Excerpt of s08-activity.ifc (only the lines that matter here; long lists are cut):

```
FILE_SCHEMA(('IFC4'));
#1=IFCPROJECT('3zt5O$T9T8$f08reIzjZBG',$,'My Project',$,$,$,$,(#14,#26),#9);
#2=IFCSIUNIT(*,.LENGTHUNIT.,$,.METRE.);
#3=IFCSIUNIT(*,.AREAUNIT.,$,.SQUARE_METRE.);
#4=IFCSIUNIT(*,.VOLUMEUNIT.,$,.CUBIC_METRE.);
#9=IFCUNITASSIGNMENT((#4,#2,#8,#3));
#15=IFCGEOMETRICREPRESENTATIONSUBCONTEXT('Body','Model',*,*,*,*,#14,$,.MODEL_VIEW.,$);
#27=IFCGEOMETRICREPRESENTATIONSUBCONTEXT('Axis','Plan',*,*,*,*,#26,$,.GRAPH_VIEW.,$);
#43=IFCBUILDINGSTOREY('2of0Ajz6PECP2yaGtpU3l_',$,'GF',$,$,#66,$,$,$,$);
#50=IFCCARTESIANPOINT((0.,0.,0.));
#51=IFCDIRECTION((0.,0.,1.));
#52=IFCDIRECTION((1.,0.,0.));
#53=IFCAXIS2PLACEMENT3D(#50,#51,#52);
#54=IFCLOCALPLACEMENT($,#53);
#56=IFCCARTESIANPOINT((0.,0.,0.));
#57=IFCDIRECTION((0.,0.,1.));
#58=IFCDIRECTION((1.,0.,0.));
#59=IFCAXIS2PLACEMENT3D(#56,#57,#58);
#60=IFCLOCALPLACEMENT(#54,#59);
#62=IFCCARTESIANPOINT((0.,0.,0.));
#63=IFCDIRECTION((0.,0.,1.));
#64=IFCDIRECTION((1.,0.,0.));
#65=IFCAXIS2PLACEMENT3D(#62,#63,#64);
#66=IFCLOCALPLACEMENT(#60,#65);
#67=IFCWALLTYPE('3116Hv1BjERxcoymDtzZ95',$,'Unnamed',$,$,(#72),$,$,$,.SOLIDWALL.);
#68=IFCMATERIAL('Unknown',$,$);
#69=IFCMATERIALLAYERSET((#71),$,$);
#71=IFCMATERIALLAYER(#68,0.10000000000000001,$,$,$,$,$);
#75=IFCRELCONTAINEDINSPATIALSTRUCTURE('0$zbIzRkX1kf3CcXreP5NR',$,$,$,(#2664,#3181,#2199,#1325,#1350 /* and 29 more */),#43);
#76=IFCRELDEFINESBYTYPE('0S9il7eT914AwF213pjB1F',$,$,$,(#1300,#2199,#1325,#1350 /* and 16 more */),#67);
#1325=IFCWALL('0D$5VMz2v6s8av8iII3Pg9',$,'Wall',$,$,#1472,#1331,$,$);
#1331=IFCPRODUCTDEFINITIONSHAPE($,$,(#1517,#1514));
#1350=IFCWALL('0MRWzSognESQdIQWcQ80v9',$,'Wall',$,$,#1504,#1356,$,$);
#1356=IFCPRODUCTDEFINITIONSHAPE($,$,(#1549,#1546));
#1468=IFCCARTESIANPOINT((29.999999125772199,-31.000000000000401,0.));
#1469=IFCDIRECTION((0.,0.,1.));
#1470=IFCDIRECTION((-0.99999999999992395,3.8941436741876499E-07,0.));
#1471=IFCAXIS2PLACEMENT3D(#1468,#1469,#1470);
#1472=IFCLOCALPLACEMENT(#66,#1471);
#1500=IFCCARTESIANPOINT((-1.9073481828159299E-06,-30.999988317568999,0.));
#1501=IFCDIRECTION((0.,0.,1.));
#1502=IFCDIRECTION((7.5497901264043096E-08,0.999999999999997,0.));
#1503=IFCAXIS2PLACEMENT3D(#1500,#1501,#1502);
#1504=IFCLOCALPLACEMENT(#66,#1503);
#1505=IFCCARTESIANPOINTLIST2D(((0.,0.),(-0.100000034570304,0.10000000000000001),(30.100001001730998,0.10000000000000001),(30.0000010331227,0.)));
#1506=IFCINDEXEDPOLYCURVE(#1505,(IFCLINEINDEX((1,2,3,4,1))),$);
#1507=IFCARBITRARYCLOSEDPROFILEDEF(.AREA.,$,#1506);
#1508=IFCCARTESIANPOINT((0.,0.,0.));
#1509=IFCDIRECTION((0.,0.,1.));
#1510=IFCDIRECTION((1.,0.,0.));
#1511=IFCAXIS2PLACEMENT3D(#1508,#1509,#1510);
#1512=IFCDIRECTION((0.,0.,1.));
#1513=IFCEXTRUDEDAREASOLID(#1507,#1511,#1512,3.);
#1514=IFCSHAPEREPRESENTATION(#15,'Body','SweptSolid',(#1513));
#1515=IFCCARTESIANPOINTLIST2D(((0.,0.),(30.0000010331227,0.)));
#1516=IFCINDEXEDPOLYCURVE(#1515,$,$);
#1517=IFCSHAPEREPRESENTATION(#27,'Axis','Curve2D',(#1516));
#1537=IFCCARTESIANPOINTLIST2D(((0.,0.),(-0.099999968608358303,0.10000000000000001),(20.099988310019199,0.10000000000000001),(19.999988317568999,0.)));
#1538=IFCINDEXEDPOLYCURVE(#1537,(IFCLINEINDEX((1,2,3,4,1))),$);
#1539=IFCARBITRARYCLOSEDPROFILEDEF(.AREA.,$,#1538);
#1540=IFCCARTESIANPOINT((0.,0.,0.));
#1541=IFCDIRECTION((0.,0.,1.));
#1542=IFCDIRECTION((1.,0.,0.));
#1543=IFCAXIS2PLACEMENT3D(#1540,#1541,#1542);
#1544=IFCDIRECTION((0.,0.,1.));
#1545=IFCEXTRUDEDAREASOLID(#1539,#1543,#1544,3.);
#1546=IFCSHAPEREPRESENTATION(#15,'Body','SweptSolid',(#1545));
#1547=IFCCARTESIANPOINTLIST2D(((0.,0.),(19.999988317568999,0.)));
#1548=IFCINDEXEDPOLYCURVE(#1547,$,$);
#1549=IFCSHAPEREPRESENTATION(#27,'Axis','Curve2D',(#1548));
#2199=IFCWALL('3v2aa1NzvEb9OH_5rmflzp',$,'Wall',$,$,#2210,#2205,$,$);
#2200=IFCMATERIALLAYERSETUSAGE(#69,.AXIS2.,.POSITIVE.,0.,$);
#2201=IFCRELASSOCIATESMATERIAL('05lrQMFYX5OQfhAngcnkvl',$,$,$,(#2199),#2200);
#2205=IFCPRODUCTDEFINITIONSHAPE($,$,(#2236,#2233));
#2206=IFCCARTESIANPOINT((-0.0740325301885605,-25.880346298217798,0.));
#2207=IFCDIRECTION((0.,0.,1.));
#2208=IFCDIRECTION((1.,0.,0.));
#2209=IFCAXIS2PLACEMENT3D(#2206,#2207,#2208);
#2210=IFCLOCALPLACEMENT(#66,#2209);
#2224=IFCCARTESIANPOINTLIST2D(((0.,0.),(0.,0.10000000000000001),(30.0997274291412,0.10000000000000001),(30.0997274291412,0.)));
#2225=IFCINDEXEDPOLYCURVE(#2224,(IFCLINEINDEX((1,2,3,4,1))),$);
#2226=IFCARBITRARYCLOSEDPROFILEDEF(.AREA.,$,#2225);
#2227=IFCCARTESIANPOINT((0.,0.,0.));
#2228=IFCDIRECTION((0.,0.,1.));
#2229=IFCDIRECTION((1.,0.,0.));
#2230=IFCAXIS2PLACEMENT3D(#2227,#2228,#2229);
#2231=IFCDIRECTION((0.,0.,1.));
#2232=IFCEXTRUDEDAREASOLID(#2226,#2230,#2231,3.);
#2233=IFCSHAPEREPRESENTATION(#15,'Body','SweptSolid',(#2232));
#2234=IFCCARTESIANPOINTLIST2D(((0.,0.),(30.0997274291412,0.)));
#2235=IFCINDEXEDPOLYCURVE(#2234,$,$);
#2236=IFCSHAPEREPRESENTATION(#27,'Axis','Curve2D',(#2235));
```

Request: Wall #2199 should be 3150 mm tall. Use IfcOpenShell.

```python
import ifcopenshell
import ifcopenshell.geom
import ifcopenshell.util.representation
import ifcopenshell.util.shape
import ifcopenshell.util.unit

model = ifcopenshell.open("s08-activity.ifc")
unit_scale = ifcopenshell.util.unit.calculate_unit_scale(model)
settings = ifcopenshell.geom.settings()


def volume(element):
    """Net volume in cubic metres, openings subtracted."""
    shape = ifcopenshell.geom.create_shape(settings, element)
    return ifcopenshell.util.shape.get_volume(shape.geometry)


wall = model.by_guid("3v2aa1NzvEb9OH_5rmflzp")
before = volume(wall)

body = ifcopenshell.util.representation.get_representation(wall, "Model", "Body")
solid = body.Items[0]
old_height = solid.Depth
solid.Depth = 3.15 / unit_scale
after = volume(wall)

print(f"height {old_height:g} -> {solid.Depth:g}, volume {before:.3f} -> {after:.3f} m3")

model.write("s08-activity-out.ifc")
```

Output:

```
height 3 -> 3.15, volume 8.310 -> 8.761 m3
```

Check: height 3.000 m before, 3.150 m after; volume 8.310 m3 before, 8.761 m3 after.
